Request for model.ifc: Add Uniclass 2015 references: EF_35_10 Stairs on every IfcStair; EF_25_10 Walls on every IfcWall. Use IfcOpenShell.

First a look at what the model holds.

```python
import ifcopenshell

model = ifcopenshell.open("model.ifc")
print(model.schema)
print("classifications:", [c.Name for c in model.by_type("IfcClassification")])
for ifc_class in ("IfcDoor", "IfcRoof", "IfcStair", "IfcWall", "IfcWindow"):
    print(ifc_class, len(model.by_type(ifc_class)))
```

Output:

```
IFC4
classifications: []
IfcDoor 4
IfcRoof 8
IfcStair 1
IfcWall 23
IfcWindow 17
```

```python
import ifcopenshell
import ifcopenshell.api.classification

model = ifcopenshell.open("model.ifc")

system = ifcopenshell.api.classification.add_classification(model, classification="Uniclass 2015")

codes = {
    "IfcStair": ("EF_35_10", "Stairs"),
    "IfcWall": ("EF_25_10", "Walls"),
}
for ifc_class, (code, name) in codes.items():
    products = model.by_type(ifc_class)
    ifcopenshell.api.classification.add_reference(
        model, products=products, classification=system, identification=code, name=name
    )
    print(code, len(products))

model.write("model_rev.ifc")
```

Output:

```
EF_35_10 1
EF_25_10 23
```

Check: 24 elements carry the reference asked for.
